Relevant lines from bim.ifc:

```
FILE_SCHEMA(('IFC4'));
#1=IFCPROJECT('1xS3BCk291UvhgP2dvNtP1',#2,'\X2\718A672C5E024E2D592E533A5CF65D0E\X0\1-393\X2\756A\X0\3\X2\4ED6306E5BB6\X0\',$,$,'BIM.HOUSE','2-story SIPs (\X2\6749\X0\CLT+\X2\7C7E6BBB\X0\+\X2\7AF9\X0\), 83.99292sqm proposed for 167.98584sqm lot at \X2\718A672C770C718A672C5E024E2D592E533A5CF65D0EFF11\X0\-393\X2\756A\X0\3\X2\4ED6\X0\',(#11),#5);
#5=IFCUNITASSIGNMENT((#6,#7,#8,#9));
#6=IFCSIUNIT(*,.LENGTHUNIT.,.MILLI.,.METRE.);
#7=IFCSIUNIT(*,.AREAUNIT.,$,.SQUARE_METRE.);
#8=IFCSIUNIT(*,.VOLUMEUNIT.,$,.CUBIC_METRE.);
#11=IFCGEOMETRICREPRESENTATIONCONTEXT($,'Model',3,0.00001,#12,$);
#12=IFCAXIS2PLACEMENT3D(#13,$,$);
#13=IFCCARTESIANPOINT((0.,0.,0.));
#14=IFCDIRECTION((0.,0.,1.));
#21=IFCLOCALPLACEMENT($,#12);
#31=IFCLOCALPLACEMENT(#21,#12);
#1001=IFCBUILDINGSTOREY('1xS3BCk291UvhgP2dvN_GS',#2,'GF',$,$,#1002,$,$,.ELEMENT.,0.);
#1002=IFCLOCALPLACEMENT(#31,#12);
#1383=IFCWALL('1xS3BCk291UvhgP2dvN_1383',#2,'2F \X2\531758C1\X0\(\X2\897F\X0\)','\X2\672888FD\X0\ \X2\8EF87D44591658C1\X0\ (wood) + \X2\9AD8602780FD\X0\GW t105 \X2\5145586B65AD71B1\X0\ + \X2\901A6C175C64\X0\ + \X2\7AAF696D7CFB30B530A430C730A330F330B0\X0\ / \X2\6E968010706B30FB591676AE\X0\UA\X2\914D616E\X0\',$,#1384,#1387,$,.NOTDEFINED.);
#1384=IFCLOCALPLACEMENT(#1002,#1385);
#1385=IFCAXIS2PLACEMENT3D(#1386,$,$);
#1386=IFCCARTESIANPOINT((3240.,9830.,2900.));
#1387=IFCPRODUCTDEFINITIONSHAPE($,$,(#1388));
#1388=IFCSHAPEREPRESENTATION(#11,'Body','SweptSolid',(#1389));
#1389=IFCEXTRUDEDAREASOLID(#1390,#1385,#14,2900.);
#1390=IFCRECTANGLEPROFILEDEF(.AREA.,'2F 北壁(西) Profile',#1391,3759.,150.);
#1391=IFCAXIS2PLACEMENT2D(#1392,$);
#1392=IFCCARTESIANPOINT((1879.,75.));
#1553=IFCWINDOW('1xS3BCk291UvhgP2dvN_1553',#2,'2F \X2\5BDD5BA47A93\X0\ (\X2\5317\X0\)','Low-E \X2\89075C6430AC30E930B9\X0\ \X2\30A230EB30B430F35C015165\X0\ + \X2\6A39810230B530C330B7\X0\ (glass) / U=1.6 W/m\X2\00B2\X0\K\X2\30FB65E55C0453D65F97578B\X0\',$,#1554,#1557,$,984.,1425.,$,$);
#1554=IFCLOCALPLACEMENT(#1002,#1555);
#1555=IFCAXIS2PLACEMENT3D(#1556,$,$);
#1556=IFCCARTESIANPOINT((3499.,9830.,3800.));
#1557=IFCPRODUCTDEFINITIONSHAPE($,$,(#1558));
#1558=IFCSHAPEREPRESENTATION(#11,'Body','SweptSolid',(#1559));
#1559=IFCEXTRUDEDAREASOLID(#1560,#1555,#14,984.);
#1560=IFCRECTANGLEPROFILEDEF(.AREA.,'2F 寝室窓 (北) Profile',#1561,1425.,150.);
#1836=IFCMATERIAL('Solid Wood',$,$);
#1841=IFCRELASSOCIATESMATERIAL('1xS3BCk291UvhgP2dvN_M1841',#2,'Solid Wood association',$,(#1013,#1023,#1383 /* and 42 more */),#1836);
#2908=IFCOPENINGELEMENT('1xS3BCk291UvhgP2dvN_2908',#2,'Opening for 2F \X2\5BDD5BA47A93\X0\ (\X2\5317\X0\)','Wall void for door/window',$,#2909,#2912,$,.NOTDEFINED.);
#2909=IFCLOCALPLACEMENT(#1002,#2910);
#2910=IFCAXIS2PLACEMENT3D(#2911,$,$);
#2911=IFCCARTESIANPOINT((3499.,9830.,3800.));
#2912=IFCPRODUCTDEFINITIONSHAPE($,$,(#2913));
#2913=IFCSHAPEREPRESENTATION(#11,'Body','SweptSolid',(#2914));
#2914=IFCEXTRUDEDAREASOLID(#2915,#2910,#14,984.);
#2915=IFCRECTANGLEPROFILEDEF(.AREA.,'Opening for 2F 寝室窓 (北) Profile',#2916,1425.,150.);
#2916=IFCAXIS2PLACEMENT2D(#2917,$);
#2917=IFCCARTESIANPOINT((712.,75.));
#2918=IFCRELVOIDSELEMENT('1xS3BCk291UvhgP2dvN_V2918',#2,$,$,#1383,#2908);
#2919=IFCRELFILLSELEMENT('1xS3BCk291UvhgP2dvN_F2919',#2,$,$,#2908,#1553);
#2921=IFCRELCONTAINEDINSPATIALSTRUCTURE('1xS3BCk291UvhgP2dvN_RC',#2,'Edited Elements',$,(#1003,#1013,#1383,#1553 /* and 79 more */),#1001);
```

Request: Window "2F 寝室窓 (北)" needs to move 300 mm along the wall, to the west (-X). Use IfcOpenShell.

```python
import ifcopenshell
import ifcopenshell.api.geometry
import ifcopenshell.util.placement

model = ifcopenshell.open("bim.ifc")

window = model.by_guid("1xS3BCk291UvhgP2dvN_1553")
opening = window.FillsVoids[0].RelatingOpeningElement
wall = opening.VoidsElements[0].RelatingBuildingElement

wall_matrix = ifcopenshell.util.placement.get_local_placement(wall.ObjectPlacement)
shift = wall_matrix[:3, 0] * -300.0
before = ifcopenshell.util.placement.get_local_placement(window.ObjectPlacement)[:3, 3].copy()

# The window is not placed relative to its opening, so move both.
for product in (opening, window):
    matrix = ifcopenshell.util.placement.get_local_placement(product.ObjectPlacement)
    matrix[:3, 3] += shift
    ifcopenshell.api.geometry.edit_object_placement(model, product=product, matrix=matrix, is_si=False)

after = ifcopenshell.util.placement.get_local_placement(window.ObjectPlacement)[:3, 3]
print("window moved by", (after - before).round(3) + 0.0)

model.write("bim_rev.ifc")
```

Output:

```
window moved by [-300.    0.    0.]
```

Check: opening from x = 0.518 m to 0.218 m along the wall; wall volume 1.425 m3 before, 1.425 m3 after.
